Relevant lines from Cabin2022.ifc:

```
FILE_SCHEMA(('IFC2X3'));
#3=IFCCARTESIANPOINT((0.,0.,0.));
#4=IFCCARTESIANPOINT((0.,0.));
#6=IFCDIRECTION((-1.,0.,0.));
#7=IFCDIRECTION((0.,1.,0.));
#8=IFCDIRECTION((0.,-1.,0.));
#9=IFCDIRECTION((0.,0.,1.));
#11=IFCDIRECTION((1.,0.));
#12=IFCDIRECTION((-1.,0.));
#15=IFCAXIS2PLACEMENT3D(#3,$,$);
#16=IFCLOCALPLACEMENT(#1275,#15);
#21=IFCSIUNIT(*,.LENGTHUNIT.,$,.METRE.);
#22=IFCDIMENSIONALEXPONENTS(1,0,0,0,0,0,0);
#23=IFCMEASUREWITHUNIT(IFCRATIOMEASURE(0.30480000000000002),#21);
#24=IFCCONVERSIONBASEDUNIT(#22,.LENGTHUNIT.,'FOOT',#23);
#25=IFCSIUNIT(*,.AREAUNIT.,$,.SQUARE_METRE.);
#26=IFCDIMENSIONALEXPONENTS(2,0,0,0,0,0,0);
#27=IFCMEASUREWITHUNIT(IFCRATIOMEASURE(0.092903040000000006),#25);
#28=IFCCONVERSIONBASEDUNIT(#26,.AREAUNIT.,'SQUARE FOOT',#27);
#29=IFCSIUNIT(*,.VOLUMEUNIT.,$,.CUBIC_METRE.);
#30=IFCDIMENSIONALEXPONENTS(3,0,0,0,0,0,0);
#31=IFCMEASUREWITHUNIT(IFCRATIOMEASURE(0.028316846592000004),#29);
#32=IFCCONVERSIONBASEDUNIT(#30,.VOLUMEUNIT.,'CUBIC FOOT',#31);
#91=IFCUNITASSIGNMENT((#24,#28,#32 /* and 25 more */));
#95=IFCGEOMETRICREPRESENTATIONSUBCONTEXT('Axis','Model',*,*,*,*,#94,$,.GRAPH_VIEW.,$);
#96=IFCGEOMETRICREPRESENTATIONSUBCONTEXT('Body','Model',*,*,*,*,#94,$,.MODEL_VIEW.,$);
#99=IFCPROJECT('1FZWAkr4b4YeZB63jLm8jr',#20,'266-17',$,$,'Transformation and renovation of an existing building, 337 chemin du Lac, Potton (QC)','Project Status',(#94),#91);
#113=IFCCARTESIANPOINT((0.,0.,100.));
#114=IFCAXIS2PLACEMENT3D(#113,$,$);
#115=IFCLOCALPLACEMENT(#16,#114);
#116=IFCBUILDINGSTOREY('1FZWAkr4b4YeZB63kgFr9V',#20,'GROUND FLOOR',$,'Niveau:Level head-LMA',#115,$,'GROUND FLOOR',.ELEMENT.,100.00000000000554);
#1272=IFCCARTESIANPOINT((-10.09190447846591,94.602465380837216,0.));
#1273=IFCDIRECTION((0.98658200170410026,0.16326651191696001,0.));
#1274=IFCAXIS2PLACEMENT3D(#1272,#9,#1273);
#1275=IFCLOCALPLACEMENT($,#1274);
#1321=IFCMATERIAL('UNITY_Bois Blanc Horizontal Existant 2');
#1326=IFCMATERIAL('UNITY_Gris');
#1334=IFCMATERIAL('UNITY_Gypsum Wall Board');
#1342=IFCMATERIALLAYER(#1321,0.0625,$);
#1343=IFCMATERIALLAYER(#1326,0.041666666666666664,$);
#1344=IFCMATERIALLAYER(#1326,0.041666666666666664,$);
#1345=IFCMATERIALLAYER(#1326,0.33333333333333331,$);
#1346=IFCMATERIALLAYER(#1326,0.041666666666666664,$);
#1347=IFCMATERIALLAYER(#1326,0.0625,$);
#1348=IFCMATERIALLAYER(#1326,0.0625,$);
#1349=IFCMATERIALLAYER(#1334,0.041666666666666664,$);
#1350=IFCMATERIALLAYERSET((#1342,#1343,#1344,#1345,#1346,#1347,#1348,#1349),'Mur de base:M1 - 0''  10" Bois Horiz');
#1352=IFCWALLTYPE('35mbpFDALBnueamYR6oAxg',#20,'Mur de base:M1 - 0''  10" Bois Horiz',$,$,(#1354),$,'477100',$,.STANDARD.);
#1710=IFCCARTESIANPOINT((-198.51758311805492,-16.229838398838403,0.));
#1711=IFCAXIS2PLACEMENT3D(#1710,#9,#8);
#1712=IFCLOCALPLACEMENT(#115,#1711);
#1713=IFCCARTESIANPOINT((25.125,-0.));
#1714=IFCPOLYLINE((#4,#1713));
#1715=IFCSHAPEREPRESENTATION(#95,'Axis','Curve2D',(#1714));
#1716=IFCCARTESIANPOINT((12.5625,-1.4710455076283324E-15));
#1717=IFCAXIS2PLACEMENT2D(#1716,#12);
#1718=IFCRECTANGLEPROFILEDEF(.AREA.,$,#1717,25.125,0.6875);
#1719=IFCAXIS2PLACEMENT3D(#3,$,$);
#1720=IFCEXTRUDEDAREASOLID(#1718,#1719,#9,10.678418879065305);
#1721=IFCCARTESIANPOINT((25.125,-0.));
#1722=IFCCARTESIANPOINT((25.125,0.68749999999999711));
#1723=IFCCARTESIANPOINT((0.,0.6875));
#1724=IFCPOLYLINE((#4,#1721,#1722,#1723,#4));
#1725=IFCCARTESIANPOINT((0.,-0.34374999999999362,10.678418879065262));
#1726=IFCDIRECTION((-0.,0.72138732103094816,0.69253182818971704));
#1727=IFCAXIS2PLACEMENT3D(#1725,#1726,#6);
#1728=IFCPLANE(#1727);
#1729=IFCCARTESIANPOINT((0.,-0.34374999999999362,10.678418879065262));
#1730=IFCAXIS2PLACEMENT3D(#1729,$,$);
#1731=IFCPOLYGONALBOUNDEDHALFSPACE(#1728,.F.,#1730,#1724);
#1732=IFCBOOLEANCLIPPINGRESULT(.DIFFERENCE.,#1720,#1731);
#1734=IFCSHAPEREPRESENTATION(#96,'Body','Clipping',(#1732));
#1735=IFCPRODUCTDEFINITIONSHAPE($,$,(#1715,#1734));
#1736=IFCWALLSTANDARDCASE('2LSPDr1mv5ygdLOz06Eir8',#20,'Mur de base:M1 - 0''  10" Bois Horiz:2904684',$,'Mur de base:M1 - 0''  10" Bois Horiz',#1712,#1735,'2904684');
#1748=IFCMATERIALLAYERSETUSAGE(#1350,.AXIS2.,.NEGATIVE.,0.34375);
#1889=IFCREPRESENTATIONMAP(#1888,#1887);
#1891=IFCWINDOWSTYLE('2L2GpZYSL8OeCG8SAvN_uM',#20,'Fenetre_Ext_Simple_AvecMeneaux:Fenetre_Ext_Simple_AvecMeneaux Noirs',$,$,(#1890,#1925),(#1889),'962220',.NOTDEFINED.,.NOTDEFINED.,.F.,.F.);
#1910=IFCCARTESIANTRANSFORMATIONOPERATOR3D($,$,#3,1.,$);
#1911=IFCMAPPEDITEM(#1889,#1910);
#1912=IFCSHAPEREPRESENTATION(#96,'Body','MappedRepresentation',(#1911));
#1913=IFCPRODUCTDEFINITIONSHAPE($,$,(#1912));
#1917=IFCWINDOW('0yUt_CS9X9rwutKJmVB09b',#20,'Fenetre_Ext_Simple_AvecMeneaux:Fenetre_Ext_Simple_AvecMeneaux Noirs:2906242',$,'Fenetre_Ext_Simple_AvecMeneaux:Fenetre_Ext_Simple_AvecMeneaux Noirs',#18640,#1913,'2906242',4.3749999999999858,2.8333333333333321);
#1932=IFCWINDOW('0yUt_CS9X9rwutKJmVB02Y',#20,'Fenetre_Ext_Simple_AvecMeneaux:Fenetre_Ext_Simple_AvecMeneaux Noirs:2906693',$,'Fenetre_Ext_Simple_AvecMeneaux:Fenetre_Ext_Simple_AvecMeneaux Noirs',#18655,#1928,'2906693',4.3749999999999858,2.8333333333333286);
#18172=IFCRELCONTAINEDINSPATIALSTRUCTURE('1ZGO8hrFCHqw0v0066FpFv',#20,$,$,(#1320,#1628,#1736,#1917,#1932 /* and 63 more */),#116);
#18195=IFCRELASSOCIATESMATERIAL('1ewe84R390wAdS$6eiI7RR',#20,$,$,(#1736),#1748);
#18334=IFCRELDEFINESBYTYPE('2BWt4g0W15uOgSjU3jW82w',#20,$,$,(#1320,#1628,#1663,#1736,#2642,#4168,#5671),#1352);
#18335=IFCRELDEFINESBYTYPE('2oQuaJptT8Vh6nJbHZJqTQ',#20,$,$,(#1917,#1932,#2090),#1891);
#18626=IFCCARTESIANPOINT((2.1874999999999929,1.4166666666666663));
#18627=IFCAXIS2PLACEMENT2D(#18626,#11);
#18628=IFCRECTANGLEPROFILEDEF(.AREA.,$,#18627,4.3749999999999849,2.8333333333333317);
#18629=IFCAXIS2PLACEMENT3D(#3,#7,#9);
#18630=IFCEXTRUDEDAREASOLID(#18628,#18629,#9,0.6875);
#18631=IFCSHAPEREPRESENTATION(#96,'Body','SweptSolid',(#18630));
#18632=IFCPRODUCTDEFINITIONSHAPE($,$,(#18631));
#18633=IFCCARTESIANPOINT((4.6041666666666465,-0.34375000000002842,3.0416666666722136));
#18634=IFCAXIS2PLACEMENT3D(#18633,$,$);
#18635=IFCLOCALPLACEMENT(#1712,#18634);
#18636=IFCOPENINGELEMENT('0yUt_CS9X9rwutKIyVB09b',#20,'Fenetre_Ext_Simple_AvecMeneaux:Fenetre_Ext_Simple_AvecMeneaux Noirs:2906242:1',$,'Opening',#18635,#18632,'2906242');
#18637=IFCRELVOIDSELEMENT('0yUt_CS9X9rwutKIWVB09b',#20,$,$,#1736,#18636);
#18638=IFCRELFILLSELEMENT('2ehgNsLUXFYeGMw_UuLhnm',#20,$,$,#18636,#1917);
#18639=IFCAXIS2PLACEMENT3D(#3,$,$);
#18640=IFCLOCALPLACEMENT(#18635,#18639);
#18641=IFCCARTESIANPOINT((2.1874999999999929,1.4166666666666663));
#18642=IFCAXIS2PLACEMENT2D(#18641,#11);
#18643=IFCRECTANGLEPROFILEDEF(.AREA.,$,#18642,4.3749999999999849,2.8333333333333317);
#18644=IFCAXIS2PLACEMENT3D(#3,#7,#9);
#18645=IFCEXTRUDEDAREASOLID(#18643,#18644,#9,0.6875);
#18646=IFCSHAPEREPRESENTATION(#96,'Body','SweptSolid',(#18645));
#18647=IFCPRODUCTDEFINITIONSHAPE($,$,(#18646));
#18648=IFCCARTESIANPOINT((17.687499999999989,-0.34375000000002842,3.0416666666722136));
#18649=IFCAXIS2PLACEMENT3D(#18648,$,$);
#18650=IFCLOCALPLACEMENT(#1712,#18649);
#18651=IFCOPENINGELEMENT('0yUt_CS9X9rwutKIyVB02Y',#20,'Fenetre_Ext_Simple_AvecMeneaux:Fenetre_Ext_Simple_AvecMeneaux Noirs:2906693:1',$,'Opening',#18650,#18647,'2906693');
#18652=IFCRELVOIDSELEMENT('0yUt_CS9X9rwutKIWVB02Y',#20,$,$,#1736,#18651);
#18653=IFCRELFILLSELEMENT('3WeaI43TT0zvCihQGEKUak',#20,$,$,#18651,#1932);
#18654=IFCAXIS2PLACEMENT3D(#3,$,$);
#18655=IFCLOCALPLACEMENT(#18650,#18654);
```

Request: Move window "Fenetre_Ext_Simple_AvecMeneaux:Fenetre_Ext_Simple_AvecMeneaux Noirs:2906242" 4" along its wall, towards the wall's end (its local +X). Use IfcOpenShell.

```python
import ifcopenshell
import ifcopenshell.api.geometry
import ifcopenshell.util.placement
import ifcopenshell.util.unit

model = ifcopenshell.open("Cabin2022.ifc")
unit_scale = ifcopenshell.util.unit.calculate_unit_scale(model)

window = model.by_id(1917)
opening = window.FillsVoids[0].RelatingOpeningElement
wall = opening.VoidsElements[0].RelatingBuildingElement

wall_matrix = ifcopenshell.util.placement.get_local_placement(wall.ObjectPlacement)
shift = wall_matrix[:3, 0] * 4 * 0.0254 / unit_scale
before = ifcopenshell.util.placement.get_local_placement(window.ObjectPlacement)[:3, 3].copy()

# The window is placed relative to its opening, so it follows when the opening moves.
matrix = ifcopenshell.util.placement.get_local_placement(opening.ObjectPlacement)
matrix[:3, 3] += shift
ifcopenshell.api.geometry.edit_object_placement(
    model, product=opening, matrix=matrix, is_si=False, should_transform_children=True
)

after = ifcopenshell.util.placement.get_local_placement(window.ObjectPlacement)[:3, 3]
print("window moved by", (after - before).round(3) + 0.0)

model.write("Cabin2022_rev.ifc")
```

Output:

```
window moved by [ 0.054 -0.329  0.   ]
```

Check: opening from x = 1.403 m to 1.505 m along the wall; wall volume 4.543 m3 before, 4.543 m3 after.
